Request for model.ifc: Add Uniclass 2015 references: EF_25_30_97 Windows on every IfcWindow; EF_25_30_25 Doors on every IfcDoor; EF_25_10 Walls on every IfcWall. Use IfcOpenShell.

First a look at what the model holds.

```python
import ifcopenshell

model = ifcopenshell.open("model.ifc")
print(model.schema)
print("classifications:", [c.Name for c in model.by_type("IfcClassification")])
for ifc_class in ("IfcDoor", "IfcRoof", "IfcStair", "IfcWall", "IfcWindow"):
    print(ifc_class, len(model.by_type(ifc_class)))
```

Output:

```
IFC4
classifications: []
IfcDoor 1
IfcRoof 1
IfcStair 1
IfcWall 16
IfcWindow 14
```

```python
import ifcopenshell
import ifcopenshell.api.classification

model = ifcopenshell.open("model.ifc")

system = ifcopenshell.api.classification.add_classification(model, classification="Uniclass 2015")

codes = {
    "IfcWindow": ("EF_25_30_97", "Windows"),
    "IfcDoor": ("EF_25_30_25", "Doors"),
    "IfcWall": ("EF_25_10", "Walls"),
}
for ifc_class, (code, name) in codes.items():
    products = model.by_type(ifc_class)
    ifcopenshell.api.classification.add_reference(
        model, products=products, classification=system, identification=code, name=name
    )
    print(code, len(products))

model.write("model_edited.ifc")
```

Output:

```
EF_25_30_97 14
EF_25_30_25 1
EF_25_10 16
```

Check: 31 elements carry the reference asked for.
